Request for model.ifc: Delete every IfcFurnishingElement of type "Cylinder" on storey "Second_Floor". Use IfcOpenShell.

First a look at what the model holds.

```python
import ifcopenshell
import ifcopenshell.util.element

model = ifcopenshell.open("model.ifc")
print(model.schema)
storey = next(s for s in model.by_type("IfcBuildingStorey") if s.Name == "Second_Floor")
furniture = [e for e in ifcopenshell.util.element.get_decomposition(storey) if e.is_a("IfcFurnishingElement")]
seen = {}
for e in furniture:
    element_type = ifcopenshell.util.element.get_type(e)
    name = element_type.Name if element_type not in (None, e) else None
    seen[name] = seen.get(name, 0) + 1
for name, count in sorted(seen.items(), key=str):
    print(count, "x", name)
```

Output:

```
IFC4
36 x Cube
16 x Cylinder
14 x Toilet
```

```python
import ifcopenshell
import ifcopenshell.api.root
import ifcopenshell.util.element

model = ifcopenshell.open("model.ifc")

storey = next(s for s in model.by_type("IfcBuildingStorey") if s.Name == "Second_Floor")
furniture = [e for e in ifcopenshell.util.element.get_decomposition(storey) if e.is_a("IfcFurnishingElement")]
targets = [e for e in furniture if (t := ifcopenshell.util.element.get_type(e)) not in (None, e) and t.Name == "Cylinder"]

for e in targets:
    ifcopenshell.api.root.remove_product(model, product=e)
print(len(targets), "removed")

model.write("model_edited.ifc")
```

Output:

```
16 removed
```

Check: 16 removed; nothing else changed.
